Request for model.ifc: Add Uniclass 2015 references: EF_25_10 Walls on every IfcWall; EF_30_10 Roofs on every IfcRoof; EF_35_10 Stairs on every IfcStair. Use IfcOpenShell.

First a look at what the model holds.

```python
import ifcopenshell

model = ifcopenshell.open("model.ifc")
print(model.schema)
print("classifications:", [c.Name for c in model.by_type("IfcClassification")])
for ifc_class in ("IfcDoor", "IfcRoof", "IfcStair", "IfcWall", "IfcWindow"):
    print(ifc_class, len(model.by_type(ifc_class)))
```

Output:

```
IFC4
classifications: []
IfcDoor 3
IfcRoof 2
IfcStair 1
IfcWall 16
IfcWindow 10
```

```python
import ifcopenshell
import ifcopenshell.api.classification

model = ifcopenshell.open("model.ifc")

system = ifcopenshell.api.classification.add_classification(model, classification="Uniclass 2015")

codes = {
    "IfcWall": ("EF_25_10", "Walls"),
    "IfcRoof": ("EF_30_10", "Roofs"),
    "IfcStair": ("EF_35_10", "Stairs"),
}
for ifc_class, (code, name) in codes.items():
    products = model.by_type(ifc_class)
    ifcopenshell.api.classification.add_reference(
        model, products=products, classification=system, identification=code, name=name
    )
    print(code, len(products))

model.write("model-out.ifc")
```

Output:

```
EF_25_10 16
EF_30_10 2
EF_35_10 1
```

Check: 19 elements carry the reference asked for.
